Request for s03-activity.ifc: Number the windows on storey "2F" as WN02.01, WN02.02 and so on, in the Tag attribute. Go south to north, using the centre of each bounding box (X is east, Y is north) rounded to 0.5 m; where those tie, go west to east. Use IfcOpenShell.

First a look at what the model holds.

```python
import ifcopenshell
import ifcopenshell.util.element
import ifcopenshell.util.placement

model = ifcopenshell.open("s03-activity.ifc")
print(model.schema)
storey = next(s for s in model.by_type("IfcBuildingStorey") if s.Name == "2F")
windows = [e for e in ifcopenshell.util.element.get_decomposition(storey) if e.is_a("IfcWindow")]
for e in sorted(windows, key=lambda e: e.id()):
    origin = ifcopenshell.util.placement.get_local_placement(e.ObjectPlacement)[:3, 3]
    print(e.id(), e.Tag, e.Name, origin.round(2) + 0.0, sep=" | ")
```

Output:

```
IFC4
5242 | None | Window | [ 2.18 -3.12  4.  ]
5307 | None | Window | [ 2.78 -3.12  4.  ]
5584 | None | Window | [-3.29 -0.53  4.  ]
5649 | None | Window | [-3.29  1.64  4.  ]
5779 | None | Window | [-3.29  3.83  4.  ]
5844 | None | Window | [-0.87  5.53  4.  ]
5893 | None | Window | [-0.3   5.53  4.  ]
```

```python
import ifcopenshell
import ifcopenshell.geom
import ifcopenshell.util.element
import ifcopenshell.util.shape

model = ifcopenshell.open("s03-activity.ifc")
settings = ifcopenshell.geom.settings()
settings.set("use-world-coords", True)


def centre(element):
    shape = ifcopenshell.geom.create_shape(settings, element)
    return ifcopenshell.util.shape.get_bbox_centroid(shape.geometry)


storey = next(s for s in model.by_type("IfcBuildingStorey") if s.Name == "2F")
windows = [e for e in ifcopenshell.util.element.get_decomposition(storey) if e.is_a("IfcWindow")]

# Insertion points can sit at a corner or the storey origin, so sort by the geometry (in metres).
centres = {e: centre(e) for e in windows}
windows.sort(key=lambda e: (round(centres[e][1] / 0.5), centres[e][0]))

for i, e in enumerate(windows, start=1):
    number = f"WN02.{i:02d}"
    e.Tag = number
    print(e.id(), number)

model.write("s03-activity_v2.ifc")
```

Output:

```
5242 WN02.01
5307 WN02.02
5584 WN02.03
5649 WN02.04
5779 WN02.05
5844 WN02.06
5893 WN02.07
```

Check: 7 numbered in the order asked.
